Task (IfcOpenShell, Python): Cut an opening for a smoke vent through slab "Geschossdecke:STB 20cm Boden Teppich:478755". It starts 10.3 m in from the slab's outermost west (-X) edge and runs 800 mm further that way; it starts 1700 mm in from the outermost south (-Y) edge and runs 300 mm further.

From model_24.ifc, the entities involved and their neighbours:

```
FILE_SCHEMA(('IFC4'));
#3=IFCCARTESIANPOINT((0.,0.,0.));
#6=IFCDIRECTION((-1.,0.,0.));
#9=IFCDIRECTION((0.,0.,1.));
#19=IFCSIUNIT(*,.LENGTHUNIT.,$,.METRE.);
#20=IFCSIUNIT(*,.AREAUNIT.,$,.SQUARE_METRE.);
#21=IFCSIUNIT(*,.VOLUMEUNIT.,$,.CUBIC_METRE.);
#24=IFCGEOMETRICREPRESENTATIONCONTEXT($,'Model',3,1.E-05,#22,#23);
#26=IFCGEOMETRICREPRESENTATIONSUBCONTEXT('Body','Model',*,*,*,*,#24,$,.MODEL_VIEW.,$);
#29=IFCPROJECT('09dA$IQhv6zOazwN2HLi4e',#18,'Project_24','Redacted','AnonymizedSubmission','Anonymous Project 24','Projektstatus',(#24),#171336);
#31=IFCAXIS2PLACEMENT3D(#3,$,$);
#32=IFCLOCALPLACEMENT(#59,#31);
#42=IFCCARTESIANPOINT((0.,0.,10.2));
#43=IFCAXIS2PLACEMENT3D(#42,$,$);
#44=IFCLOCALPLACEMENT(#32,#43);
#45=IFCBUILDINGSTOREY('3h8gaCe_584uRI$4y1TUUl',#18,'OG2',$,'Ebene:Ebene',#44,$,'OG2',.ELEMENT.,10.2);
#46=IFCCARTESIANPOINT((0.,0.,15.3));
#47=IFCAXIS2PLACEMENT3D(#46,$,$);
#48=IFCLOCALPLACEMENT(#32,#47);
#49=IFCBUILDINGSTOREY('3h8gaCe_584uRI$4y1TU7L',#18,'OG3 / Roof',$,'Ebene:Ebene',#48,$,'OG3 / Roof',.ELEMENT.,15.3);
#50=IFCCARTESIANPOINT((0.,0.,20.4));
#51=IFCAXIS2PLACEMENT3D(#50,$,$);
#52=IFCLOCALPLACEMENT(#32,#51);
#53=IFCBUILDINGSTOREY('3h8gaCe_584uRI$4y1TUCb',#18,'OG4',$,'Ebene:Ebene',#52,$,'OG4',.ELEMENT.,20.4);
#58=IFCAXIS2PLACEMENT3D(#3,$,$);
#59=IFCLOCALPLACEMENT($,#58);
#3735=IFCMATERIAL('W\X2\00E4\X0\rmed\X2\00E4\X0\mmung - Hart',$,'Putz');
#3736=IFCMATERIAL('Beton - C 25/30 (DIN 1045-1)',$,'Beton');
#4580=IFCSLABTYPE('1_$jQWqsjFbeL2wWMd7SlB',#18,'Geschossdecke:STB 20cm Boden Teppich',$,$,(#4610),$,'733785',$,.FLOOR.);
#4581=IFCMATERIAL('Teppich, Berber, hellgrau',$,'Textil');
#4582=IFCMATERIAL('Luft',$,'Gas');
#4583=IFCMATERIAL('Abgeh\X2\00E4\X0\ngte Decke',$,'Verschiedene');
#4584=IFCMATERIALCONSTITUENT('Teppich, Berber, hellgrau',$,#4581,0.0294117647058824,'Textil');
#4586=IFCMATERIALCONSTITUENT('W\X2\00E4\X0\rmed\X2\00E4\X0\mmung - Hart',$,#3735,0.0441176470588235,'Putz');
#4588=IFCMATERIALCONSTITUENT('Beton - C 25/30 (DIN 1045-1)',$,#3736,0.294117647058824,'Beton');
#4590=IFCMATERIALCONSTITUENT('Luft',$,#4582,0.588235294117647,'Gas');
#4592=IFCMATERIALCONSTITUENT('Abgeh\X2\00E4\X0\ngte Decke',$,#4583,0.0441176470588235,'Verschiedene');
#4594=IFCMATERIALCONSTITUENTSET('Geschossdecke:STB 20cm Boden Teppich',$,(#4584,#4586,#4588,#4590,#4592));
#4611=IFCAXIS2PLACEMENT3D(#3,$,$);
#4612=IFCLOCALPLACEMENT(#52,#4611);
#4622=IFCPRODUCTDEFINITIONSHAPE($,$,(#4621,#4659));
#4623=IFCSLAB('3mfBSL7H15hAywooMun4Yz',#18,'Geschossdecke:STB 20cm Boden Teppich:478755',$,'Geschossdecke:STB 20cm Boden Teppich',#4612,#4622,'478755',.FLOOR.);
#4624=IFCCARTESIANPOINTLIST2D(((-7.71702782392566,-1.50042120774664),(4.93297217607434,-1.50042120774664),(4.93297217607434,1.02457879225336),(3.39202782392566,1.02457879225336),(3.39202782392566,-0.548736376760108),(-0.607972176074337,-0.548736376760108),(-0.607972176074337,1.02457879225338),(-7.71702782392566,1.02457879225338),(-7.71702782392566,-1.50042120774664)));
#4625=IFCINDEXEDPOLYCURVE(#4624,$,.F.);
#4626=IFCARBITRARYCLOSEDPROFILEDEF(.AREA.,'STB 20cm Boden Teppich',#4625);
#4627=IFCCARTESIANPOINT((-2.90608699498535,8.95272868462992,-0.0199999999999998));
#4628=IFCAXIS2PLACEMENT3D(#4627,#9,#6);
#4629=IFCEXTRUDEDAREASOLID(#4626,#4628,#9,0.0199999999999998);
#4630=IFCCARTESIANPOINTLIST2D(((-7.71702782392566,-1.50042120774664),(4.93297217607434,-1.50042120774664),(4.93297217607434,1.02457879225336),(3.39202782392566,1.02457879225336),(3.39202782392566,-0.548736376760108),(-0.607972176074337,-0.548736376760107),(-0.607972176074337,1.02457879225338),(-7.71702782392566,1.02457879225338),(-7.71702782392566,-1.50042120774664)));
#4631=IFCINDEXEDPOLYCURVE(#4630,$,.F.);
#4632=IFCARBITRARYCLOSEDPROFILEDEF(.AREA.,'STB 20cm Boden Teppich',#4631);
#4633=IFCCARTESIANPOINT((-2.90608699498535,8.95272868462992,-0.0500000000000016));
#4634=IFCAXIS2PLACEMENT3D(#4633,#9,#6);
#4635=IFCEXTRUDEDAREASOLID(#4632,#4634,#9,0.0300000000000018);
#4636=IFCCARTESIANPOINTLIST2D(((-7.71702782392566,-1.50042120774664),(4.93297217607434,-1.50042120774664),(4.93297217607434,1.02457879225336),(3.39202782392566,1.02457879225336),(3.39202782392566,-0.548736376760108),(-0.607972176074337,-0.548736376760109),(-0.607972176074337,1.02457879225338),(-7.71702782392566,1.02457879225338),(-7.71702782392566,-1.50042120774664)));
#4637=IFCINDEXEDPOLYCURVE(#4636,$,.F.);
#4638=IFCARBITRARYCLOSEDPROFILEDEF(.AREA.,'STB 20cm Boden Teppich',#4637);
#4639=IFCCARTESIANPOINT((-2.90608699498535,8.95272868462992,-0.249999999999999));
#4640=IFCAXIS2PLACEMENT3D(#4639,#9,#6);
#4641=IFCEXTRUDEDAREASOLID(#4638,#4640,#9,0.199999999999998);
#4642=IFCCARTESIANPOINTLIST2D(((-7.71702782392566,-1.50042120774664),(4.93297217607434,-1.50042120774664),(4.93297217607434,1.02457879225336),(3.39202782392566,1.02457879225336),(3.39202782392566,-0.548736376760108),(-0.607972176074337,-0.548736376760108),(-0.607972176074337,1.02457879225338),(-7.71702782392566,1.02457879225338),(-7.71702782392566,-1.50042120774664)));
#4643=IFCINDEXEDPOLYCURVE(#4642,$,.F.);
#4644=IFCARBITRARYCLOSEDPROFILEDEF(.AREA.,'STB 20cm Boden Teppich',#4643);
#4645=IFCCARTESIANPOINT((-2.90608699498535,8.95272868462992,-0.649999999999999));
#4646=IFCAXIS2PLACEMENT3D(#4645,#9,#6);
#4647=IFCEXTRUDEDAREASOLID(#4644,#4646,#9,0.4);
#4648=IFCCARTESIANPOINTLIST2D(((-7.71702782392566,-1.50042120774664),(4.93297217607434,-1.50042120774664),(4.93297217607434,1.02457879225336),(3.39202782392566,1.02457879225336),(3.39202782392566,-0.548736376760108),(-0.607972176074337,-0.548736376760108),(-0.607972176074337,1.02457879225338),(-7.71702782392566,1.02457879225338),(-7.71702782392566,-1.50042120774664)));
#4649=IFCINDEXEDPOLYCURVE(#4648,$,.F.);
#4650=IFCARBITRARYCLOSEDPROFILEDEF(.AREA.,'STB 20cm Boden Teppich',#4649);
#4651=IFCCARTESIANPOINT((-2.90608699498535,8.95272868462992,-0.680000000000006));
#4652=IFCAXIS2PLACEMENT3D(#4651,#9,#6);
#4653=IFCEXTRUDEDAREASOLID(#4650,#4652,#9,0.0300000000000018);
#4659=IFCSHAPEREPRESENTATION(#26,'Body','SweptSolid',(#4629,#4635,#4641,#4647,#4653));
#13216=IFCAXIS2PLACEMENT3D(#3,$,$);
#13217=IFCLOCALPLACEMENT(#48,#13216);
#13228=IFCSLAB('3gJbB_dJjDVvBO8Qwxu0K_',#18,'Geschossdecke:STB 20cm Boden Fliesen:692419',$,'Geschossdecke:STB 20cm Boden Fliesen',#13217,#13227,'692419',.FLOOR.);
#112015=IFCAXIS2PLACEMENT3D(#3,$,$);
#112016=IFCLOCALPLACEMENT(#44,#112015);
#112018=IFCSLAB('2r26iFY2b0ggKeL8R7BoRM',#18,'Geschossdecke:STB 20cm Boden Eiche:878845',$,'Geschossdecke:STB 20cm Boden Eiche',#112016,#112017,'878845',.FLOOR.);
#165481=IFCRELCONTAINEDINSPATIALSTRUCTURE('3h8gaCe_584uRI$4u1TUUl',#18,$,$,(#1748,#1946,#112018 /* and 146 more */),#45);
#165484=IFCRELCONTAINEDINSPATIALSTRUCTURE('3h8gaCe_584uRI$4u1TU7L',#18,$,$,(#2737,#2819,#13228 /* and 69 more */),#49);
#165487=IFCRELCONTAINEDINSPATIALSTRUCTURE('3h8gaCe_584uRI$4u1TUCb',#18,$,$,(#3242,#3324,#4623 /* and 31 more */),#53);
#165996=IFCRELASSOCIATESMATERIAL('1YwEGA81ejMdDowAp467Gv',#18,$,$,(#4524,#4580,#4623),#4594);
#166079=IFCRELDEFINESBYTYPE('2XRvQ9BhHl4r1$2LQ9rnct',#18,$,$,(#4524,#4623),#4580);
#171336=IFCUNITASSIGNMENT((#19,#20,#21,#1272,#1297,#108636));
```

```python
import numpy as np
import ifcopenshell
import ifcopenshell.api.feature
import ifcopenshell.api.geometry
import ifcopenshell.api.root
import ifcopenshell.geom
import ifcopenshell.util.placement
import ifcopenshell.util.representation
import ifcopenshell.util.shape
import ifcopenshell.util.unit

model = ifcopenshell.open("model_24.ifc")
unit_scale = ifcopenshell.util.unit.calculate_unit_scale(model)
settings = ifcopenshell.geom.settings()


def volume(element):
    """Net volume in cubic metres, openings subtracted."""
    shape = ifcopenshell.geom.create_shape(settings, element)
    return ifcopenshell.util.shape.get_volume(shape.geometry)


slab = model.by_id(4623)
before = volume(slab)

# Extent in the slab's own axes, in metres. The edges named are its -X and -Y sides.
slab_shape = ifcopenshell.geom.create_shape(settings, slab)
vertices = ifcopenshell.util.shape.get_vertices(slab_shape.geometry)
x_min, y_min, bottom = vertices.min(axis=0)
top = vertices[:, 2].max()

opening = ifcopenshell.api.root.create_entity(model, ifc_class="IfcOpeningElement", name="Smoke vent opening", predefined_type="OPENING")
context = ifcopenshell.util.representation.get_context(model, "Model", "Body", "MODEL_VIEW")
width, depth = 0.8, 0.3
outline = [(0.0, 0.0), (width, 0.0), (width, depth), (0.0, depth), (0.0, 0.0)]
# Overshoot both faces by 50 mm so the cut is clean.
shape = ifcopenshell.api.geometry.add_slab_representation(
    model, context=context, depth=top - bottom + 0.1, polyline=outline
)
ifcopenshell.api.geometry.assign_representation(model, product=opening, representation=shape)

matrix = ifcopenshell.util.placement.get_local_placement(slab.ObjectPlacement)
matrix[:, 3] = matrix @ np.append(np.array([x_min + 10.3, y_min + 1.7, bottom - 0.05]) / unit_scale, 1.0)
ifcopenshell.api.geometry.edit_object_placement(model, product=opening, matrix=matrix, is_si=False)
ifcopenshell.api.feature.add_feature(model, feature=opening, element=slab)

after = volume(slab)

print(f"slab volume {before:.3f} -> {after:.3f} m3")

model.write("model_24_rev.ifc")
```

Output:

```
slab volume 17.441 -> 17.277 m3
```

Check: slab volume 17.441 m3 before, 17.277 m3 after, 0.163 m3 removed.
